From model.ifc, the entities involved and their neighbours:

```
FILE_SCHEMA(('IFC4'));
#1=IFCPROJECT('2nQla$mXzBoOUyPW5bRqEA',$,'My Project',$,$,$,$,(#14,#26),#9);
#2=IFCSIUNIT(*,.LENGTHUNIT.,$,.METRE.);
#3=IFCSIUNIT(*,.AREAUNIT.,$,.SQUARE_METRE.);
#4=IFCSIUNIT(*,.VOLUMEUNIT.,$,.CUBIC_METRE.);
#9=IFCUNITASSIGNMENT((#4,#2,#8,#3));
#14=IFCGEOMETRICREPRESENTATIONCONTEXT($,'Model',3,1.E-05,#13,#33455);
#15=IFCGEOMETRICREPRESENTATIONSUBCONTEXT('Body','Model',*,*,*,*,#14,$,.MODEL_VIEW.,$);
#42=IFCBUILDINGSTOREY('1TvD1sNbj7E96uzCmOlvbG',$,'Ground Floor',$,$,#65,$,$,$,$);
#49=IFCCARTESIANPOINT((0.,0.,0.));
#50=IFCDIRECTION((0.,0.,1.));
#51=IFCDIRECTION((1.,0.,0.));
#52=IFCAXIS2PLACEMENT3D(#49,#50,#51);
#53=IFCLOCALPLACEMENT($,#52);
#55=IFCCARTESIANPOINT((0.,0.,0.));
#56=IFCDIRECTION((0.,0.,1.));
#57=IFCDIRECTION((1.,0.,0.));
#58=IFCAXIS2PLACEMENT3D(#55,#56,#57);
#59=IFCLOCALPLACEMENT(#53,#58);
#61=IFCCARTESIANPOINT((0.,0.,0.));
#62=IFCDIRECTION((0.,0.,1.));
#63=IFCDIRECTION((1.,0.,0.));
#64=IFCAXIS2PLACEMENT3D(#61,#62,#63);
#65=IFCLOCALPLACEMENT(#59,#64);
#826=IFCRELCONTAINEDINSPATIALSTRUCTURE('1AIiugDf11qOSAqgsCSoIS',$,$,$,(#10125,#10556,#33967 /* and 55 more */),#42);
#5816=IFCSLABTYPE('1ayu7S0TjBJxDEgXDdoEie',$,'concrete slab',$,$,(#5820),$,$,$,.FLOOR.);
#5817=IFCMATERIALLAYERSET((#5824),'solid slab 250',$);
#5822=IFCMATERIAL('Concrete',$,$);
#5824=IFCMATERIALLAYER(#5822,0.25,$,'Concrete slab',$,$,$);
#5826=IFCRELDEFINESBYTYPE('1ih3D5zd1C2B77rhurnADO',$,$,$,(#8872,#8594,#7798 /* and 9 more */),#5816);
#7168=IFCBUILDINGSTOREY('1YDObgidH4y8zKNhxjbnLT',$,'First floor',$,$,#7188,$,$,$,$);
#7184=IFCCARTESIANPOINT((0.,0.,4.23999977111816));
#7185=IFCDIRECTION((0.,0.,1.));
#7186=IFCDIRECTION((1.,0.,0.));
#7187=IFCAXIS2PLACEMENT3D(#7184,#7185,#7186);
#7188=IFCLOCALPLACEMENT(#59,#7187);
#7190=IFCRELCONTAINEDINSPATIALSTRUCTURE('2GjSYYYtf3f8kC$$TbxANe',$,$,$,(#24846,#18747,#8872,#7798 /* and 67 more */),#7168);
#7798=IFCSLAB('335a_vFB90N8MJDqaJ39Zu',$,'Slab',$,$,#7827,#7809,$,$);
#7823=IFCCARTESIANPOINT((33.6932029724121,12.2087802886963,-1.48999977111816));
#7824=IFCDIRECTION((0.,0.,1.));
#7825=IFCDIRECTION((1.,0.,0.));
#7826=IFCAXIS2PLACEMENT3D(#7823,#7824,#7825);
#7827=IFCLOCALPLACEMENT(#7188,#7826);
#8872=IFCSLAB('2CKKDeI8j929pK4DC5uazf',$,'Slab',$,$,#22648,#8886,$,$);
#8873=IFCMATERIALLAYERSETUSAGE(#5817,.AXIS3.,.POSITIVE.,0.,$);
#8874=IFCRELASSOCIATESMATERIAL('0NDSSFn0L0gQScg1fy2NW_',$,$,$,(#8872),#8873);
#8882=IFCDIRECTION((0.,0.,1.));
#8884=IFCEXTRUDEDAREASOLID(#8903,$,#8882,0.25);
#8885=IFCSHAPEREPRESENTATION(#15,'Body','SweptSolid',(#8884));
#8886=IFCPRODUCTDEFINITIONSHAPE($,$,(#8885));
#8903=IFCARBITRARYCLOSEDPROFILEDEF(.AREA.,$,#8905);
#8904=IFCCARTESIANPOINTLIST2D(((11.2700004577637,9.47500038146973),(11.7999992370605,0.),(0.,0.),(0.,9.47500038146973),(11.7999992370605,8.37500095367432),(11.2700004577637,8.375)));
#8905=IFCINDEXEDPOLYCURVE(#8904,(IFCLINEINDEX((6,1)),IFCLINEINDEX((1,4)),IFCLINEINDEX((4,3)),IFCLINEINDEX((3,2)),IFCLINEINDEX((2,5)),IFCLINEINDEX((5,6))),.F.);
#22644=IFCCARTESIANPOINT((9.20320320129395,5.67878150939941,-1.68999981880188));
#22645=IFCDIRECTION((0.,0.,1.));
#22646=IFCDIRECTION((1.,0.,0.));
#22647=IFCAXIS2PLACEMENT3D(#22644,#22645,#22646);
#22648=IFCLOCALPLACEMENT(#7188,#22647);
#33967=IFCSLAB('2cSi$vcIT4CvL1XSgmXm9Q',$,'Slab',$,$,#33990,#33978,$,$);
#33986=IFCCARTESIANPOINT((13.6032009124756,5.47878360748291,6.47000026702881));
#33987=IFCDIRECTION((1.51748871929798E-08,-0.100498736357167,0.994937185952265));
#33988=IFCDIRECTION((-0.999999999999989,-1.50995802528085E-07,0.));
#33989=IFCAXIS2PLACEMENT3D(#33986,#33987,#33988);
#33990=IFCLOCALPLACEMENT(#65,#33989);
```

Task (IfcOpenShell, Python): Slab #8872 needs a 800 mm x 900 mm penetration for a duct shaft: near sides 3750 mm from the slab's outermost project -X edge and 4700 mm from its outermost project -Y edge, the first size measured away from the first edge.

```python
import numpy as np
import ifcopenshell
import ifcopenshell.api.feature
import ifcopenshell.api.geometry
import ifcopenshell.api.root
import ifcopenshell.geom
import ifcopenshell.util.placement
import ifcopenshell.util.representation
import ifcopenshell.util.shape
import ifcopenshell.util.unit

model = ifcopenshell.open("model.ifc")
unit_scale = ifcopenshell.util.unit.calculate_unit_scale(model)
settings = ifcopenshell.geom.settings()


def volume(element):
    """Net volume in cubic metres, openings subtracted."""
    shape = ifcopenshell.geom.create_shape(settings, element)
    return ifcopenshell.util.shape.get_volume(shape.geometry)


slab = model.by_id(8872)
before = volume(slab)

# Extent in the slab's own axes, in metres. The edges named are its -X and -Y sides.
slab_shape = ifcopenshell.geom.create_shape(settings, slab)
vertices = ifcopenshell.util.shape.get_vertices(slab_shape.geometry)
x_min, y_min, bottom = vertices.min(axis=0)
top = vertices[:, 2].max()

opening = ifcopenshell.api.root.create_entity(model, ifc_class="IfcOpeningElement", name="Duct shaft opening", predefined_type="OPENING")
context = ifcopenshell.util.representation.get_context(model, "Model", "Body", "MODEL_VIEW")
width, depth = 0.8, 0.9
outline = [(0.0, 0.0), (width, 0.0), (width, depth), (0.0, depth), (0.0, 0.0)]
# Overshoot both faces by 50 mm so the cut is clean.
shape = ifcopenshell.api.geometry.add_slab_representation(
    model, context=context, depth=top - bottom + 0.1, polyline=outline
)
ifcopenshell.api.geometry.assign_representation(model, product=opening, representation=shape)

matrix = ifcopenshell.util.placement.get_local_placement(slab.ObjectPlacement)
matrix[:, 3] = matrix @ np.append(np.array([x_min + 3.75, y_min + 4.7, bottom - 0.05]) / unit_scale, 1.0)
ifcopenshell.api.geometry.edit_object_placement(model, product=opening, matrix=matrix, is_si=False)
ifcopenshell.api.feature.add_feature(model, feature=opening, element=slab)

after = volume(slab)

print(f"slab volume {before:.3f} -> {after:.3f} m3")

model.write("model_rev.ifc")
```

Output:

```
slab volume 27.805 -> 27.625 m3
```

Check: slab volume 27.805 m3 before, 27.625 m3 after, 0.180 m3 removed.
